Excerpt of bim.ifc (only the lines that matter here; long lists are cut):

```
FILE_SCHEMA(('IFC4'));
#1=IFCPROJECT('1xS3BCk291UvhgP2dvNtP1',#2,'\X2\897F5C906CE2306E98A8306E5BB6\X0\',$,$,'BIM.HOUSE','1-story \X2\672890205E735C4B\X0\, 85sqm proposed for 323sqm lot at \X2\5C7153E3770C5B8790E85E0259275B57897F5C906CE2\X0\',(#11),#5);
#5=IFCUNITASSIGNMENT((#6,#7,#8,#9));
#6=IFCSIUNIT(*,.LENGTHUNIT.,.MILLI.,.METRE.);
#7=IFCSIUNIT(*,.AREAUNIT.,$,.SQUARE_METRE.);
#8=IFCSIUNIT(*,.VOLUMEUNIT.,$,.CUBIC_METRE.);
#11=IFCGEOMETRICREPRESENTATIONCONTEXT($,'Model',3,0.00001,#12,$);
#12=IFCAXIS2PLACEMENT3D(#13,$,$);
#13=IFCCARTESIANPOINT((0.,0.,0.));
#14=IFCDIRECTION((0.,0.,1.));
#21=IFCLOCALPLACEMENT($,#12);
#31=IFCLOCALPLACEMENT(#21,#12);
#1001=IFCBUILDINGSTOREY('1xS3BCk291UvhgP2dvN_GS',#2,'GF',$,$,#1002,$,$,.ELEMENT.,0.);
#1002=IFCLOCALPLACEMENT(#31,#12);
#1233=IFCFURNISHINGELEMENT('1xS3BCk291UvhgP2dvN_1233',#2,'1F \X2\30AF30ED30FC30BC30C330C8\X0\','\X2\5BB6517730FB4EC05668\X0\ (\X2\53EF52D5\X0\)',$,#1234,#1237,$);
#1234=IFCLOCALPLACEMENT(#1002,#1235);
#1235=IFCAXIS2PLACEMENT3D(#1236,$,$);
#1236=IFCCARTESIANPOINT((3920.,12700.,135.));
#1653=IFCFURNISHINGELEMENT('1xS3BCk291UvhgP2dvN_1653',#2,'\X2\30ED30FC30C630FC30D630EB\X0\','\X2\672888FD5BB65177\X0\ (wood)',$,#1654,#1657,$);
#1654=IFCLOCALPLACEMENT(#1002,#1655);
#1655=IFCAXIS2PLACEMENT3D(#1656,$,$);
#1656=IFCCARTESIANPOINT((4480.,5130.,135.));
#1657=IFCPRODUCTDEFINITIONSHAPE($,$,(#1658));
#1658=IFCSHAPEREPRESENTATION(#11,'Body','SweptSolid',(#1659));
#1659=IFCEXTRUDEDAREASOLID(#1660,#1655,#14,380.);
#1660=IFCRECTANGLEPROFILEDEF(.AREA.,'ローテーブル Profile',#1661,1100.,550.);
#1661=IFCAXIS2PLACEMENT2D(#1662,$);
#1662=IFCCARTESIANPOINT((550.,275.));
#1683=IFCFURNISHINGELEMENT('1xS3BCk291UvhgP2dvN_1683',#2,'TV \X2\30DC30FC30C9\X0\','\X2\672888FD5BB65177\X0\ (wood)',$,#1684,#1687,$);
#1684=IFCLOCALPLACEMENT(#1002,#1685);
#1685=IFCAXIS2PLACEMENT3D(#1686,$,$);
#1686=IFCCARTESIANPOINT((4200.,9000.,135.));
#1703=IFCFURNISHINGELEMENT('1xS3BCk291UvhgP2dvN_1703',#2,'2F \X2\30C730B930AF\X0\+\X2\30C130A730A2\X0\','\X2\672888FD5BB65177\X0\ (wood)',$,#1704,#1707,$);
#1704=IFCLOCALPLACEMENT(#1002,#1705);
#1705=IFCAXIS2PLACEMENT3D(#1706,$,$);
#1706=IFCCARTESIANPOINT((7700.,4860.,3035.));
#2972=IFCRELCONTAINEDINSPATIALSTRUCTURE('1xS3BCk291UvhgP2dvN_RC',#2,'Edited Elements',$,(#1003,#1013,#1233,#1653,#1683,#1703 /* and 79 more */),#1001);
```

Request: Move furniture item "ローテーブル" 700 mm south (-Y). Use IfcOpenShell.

```python
import ifcopenshell
import ifcopenshell.api.geometry
import ifcopenshell.util.placement
import ifcopenshell.util.unit

model = ifcopenshell.open("bim.ifc")
unit_scale = ifcopenshell.util.unit.calculate_unit_scale(model)

item = model.by_id(1653)
matrix = ifcopenshell.util.placement.get_local_placement(item.ObjectPlacement)
matrix[1, 3] -= 0.7 / unit_scale
ifcopenshell.api.geometry.edit_object_placement(model, product=item, matrix=matrix, is_si=False)

print(ifcopenshell.util.placement.get_local_placement(item.ObjectPlacement).round(3) + 0.0)

model.write("bim_v2.ifc")
```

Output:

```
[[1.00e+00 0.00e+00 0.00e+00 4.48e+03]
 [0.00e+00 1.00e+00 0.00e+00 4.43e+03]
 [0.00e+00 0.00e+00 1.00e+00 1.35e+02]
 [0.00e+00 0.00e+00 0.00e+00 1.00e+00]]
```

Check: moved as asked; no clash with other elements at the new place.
